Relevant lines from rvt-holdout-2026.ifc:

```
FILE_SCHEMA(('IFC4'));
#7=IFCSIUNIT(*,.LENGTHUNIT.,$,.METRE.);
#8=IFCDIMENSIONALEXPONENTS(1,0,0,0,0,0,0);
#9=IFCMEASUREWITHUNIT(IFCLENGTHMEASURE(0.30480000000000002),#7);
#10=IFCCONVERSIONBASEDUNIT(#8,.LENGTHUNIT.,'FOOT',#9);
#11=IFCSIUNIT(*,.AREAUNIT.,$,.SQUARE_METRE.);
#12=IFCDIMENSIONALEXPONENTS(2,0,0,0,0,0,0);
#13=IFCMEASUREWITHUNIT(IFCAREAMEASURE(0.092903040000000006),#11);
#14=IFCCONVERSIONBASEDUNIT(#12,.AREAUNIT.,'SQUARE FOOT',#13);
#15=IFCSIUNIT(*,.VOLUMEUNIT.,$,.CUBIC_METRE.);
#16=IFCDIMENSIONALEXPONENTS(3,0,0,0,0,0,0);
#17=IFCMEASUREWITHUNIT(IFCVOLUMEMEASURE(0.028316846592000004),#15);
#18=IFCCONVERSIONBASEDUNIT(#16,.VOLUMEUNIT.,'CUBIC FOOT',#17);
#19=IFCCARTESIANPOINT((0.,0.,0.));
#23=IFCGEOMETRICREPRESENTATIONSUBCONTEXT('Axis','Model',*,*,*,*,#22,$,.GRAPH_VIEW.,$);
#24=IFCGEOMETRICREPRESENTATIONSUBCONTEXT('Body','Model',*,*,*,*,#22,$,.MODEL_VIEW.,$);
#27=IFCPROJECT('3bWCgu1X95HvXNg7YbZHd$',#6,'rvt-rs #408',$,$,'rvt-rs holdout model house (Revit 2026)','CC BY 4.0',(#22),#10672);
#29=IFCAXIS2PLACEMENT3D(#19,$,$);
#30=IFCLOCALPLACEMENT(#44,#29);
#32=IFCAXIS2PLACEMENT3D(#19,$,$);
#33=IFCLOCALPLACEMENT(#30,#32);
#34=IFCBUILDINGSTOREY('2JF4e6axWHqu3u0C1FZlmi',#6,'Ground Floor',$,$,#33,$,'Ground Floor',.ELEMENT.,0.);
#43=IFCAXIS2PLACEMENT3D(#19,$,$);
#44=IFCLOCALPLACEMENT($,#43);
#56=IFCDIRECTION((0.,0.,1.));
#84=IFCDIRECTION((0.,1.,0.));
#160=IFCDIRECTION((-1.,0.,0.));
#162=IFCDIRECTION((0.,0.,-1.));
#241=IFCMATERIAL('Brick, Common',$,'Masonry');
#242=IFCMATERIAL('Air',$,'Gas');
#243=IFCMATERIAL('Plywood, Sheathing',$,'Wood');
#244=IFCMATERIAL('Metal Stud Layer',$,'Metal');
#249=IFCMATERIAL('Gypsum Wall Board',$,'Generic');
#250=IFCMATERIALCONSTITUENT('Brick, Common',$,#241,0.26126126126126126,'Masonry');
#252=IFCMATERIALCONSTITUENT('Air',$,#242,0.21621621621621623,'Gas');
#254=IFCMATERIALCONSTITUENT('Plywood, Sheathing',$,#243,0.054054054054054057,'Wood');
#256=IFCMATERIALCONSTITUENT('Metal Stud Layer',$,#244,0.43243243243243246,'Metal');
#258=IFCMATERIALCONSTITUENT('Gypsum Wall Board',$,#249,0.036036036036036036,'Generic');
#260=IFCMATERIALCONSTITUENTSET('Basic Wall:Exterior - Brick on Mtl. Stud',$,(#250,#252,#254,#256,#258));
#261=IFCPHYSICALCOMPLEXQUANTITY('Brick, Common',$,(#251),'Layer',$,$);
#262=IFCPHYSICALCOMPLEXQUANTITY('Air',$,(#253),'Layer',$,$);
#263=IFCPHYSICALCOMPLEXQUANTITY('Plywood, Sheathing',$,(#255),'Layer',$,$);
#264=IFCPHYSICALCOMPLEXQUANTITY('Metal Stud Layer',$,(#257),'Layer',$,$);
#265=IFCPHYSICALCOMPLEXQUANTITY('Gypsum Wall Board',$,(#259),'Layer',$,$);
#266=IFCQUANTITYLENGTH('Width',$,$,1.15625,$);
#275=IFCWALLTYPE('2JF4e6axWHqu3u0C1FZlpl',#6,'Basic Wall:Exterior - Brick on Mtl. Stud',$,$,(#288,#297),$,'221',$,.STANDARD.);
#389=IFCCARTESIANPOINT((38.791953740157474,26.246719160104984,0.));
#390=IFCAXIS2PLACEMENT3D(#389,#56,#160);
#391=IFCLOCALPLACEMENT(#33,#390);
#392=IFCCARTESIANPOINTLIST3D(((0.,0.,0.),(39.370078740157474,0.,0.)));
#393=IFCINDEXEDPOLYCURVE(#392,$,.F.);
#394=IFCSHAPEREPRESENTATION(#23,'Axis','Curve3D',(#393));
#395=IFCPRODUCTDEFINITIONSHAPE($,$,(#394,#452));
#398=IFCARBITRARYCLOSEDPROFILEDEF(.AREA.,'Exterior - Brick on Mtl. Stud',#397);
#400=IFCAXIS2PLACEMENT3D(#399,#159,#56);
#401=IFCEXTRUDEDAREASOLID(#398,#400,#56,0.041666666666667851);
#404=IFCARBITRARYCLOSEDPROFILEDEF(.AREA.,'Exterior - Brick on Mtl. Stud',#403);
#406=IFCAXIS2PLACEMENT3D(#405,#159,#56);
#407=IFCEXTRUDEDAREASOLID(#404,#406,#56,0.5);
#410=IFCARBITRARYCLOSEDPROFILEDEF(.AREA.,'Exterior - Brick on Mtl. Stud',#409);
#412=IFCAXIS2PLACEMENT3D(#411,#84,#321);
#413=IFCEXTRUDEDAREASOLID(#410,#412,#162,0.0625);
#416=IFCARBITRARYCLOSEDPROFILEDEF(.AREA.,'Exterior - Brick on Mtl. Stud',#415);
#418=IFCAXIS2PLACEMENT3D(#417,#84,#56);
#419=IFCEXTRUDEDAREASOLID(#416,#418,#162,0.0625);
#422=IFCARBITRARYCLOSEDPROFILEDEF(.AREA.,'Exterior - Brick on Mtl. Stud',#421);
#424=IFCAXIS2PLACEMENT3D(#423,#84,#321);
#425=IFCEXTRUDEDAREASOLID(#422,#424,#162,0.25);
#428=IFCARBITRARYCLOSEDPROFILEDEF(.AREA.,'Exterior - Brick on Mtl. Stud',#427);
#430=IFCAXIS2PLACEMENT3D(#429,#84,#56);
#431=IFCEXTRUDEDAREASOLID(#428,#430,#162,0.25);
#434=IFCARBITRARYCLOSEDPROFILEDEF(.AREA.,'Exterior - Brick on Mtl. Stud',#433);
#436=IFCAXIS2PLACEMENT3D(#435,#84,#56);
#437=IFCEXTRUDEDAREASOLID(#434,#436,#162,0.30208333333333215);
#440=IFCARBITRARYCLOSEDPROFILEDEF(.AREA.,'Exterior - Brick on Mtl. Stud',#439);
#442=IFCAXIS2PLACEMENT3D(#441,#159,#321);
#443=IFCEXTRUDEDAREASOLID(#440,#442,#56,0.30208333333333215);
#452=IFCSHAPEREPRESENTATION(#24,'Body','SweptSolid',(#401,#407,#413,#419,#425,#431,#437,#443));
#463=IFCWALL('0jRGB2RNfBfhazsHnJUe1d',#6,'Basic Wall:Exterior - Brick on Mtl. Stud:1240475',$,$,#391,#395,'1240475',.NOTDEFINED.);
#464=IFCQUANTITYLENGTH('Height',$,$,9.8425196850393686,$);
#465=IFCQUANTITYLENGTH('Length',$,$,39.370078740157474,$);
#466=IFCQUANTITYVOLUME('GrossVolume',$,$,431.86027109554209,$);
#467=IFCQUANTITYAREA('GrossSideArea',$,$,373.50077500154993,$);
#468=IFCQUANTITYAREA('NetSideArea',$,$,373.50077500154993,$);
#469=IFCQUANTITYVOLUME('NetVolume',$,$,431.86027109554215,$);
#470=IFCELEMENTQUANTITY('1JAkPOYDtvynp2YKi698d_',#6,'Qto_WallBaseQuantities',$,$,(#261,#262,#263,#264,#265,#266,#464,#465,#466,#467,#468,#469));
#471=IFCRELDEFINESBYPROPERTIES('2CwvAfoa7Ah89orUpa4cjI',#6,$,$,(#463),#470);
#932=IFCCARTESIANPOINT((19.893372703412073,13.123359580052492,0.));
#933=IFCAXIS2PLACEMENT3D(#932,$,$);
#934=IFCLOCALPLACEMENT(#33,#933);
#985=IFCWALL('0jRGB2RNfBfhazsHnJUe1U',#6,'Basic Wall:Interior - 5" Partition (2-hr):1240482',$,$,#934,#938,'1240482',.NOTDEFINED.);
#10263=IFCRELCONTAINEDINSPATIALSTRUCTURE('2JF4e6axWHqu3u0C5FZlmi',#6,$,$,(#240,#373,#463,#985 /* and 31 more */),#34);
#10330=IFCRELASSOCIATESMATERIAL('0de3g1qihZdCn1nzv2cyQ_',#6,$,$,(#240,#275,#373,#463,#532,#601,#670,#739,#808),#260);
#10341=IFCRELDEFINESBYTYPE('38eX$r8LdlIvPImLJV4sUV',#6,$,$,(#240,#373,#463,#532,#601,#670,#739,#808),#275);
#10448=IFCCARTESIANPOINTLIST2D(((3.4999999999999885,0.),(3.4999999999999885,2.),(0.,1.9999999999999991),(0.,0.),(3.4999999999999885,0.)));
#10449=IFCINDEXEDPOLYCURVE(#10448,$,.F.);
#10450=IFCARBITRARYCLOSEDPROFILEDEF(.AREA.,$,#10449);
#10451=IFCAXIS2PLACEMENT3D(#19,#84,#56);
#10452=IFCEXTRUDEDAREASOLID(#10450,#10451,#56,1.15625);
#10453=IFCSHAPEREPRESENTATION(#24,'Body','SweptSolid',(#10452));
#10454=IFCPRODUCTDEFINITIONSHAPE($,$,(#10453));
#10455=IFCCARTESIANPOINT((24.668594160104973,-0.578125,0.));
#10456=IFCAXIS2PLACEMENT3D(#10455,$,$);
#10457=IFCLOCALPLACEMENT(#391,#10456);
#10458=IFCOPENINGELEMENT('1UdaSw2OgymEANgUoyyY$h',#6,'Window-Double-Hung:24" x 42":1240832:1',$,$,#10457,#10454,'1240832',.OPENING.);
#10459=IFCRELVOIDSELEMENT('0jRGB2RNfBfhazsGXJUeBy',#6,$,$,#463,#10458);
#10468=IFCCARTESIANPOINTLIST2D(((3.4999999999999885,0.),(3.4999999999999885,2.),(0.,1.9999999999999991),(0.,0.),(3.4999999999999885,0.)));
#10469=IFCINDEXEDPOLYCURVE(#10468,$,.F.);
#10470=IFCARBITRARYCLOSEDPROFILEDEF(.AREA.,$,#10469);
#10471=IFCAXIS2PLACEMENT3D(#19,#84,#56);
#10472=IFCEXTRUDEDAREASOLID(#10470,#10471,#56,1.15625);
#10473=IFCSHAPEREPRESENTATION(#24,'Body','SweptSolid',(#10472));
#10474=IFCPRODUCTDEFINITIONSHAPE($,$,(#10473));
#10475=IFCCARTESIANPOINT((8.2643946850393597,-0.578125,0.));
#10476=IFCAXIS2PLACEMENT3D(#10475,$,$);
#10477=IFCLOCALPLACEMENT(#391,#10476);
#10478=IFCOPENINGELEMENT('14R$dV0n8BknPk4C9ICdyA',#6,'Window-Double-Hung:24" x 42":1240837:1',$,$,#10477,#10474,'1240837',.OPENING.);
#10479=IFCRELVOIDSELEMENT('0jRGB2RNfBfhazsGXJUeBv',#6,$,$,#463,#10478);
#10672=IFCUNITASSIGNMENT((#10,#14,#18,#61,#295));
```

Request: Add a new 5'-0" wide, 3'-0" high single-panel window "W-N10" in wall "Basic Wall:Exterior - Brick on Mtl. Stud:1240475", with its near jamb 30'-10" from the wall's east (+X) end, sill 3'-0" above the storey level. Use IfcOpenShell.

```python
import numpy as np
import ifcopenshell
import ifcopenshell.api.feature
import ifcopenshell.api.geometry
import ifcopenshell.api.pset
import ifcopenshell.api.root
import ifcopenshell.api.spatial
import ifcopenshell.geom
import ifcopenshell.util.element
import ifcopenshell.util.placement
import ifcopenshell.util.representation
import ifcopenshell.util.shape
import ifcopenshell.util.unit

model = ifcopenshell.open("rvt-holdout-2026.ifc")
unit_scale = ifcopenshell.util.unit.calculate_unit_scale(model)
area_scale = ifcopenshell.util.unit.calculate_unit_scale(model, "AREAUNIT")
volume_scale = ifcopenshell.util.unit.calculate_unit_scale(model, "VOLUMEUNIT")
settings = ifcopenshell.geom.settings()


def volume(element):
    """Net volume in cubic metres, openings subtracted."""
    shape = ifcopenshell.geom.create_shape(settings, element)
    return ifcopenshell.util.shape.get_volume(shape.geometry)


wall = model.by_id(463)
storey = ifcopenshell.util.element.get_container(wall, ifc_class="IfcBuildingStorey")
context = ifcopenshell.util.representation.get_context(model, "Model", "Body", "MODEL_VIEW")
before = volume(wall)

width, height, from_end, sill = 1.524, 0.9144, 9.398, 0.9144  # metres

# The wall runs along its own X axis, and the end named is its -X end.
wall_shape = ifcopenshell.geom.create_shape(settings, wall)
x, y, z = ifcopenshell.util.shape.get_vertices(wall_shape.geometry).T
start = x.min() + from_end
face, thickness = float(y.min()), float(y.max() - y.min())
wall_matrix = ifcopenshell.util.placement.get_local_placement(wall.ObjectPlacement)
level = ifcopenshell.util.placement.get_local_placement(storey.ObjectPlacement)[2, 3]


def in_wall(x, y):
    """Placement at x, y metres in the wall's axes, at sill height."""
    matrix = wall_matrix.copy()
    matrix[:, 3] = wall_matrix @ np.array([x / unit_scale, y / unit_scale, 0.0, 1.0])
    matrix[2, 3] = level + sill / unit_scale
    return matrix


# Opening: a box that overshoots both wall faces by 50 mm.
opening = ifcopenshell.api.root.create_entity(model, ifc_class="IfcOpeningElement", predefined_type="OPENING")
box = ifcopenshell.api.geometry.add_wall_representation(
    model, context=context, length=width, height=height, thickness=thickness + 0.1
)
ifcopenshell.api.geometry.assign_representation(model, product=opening, representation=box)
ifcopenshell.api.geometry.edit_object_placement(model, product=opening, matrix=in_wall(start, face - 0.05), is_si=False)
ifcopenshell.api.feature.add_feature(model, feature=opening, element=wall)

window = ifcopenshell.api.root.create_entity(model, ifc_class="IfcWindow", name="W-N10", predefined_type="WINDOW")
window.OverallWidth, window.OverallHeight = width / unit_scale, height / unit_scale
window.PartitioningType = "SINGLE_PANEL"
body = ifcopenshell.api.geometry.add_window_representation(
    model,
    context=context,
    overall_width=window.OverallWidth,
    overall_height=window.OverallHeight,
    partition_type="SINGLE_PANEL",
)
ifcopenshell.api.geometry.assign_representation(model, product=window, representation=body)
ifcopenshell.api.spatial.assign_container(model, products=[window], relating_structure=storey)
ifcopenshell.api.feature.add_filling(model, opening=opening, element=window)

# Centre the window in the wall's thickness.
ifcopenshell.api.geometry.edit_object_placement(model, product=window, matrix=in_wall(start, face), is_si=False)
window_shape = ifcopenshell.geom.create_shape(settings, window)
depth = ifcopenshell.util.shape.get_vertices(window_shape.geometry)[:, 1]
offset = face + thickness / 2 - (depth.min() + depth.max()) / 2
ifcopenshell.api.geometry.edit_object_placement(model, product=window, matrix=in_wall(start, offset), is_si=False)

after = volume(wall)

# Update the wall's stored quantities.
qto = model.by_id(ifcopenshell.util.element.get_pset(wall, "Qto_WallBaseQuantities", should_inherit=False)["id"])
ifcopenshell.api.pset.edit_qto(model, qto=qto, properties={
    "NetSideArea": after / thickness / area_scale,
    "NetVolume": after / volume_scale,
})

print(f"wall volume {before:.3f} -> {after:.3f} m3")

model.write("rvt-holdout-2026_updated.ifc")
```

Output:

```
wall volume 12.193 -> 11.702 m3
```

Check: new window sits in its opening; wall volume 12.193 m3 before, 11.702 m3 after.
